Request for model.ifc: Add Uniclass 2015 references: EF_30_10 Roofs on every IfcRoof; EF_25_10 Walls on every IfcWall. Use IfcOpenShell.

First a look at what the model holds.

```python
import ifcopenshell

model = ifcopenshell.open("model.ifc")
print(model.schema)
print("classifications:", [c.Name for c in model.by_type("IfcClassification")])
for ifc_class in ("IfcDoor", "IfcRoof", "IfcStair", "IfcWall", "IfcWindow"):
    print(ifc_class, len(model.by_type(ifc_class)))
```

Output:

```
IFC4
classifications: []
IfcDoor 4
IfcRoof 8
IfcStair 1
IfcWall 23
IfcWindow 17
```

```python
import ifcopenshell
import ifcopenshell.api.classification

model = ifcopenshell.open("model.ifc")

system = ifcopenshell.api.classification.add_classification(model, classification="Uniclass 2015")

codes = {
    "IfcRoof": ("EF_30_10", "Roofs"),
    "IfcWall": ("EF_25_10", "Walls"),
}
for ifc_class, (code, name) in codes.items():
    products = model.by_type(ifc_class)
    ifcopenshell.api.classification.add_reference(
        model, products=products, classification=system, identification=code, name=name
    )
    print(code, len(products))

model.write("model_v2.ifc")
```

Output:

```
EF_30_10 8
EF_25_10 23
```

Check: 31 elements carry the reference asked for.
